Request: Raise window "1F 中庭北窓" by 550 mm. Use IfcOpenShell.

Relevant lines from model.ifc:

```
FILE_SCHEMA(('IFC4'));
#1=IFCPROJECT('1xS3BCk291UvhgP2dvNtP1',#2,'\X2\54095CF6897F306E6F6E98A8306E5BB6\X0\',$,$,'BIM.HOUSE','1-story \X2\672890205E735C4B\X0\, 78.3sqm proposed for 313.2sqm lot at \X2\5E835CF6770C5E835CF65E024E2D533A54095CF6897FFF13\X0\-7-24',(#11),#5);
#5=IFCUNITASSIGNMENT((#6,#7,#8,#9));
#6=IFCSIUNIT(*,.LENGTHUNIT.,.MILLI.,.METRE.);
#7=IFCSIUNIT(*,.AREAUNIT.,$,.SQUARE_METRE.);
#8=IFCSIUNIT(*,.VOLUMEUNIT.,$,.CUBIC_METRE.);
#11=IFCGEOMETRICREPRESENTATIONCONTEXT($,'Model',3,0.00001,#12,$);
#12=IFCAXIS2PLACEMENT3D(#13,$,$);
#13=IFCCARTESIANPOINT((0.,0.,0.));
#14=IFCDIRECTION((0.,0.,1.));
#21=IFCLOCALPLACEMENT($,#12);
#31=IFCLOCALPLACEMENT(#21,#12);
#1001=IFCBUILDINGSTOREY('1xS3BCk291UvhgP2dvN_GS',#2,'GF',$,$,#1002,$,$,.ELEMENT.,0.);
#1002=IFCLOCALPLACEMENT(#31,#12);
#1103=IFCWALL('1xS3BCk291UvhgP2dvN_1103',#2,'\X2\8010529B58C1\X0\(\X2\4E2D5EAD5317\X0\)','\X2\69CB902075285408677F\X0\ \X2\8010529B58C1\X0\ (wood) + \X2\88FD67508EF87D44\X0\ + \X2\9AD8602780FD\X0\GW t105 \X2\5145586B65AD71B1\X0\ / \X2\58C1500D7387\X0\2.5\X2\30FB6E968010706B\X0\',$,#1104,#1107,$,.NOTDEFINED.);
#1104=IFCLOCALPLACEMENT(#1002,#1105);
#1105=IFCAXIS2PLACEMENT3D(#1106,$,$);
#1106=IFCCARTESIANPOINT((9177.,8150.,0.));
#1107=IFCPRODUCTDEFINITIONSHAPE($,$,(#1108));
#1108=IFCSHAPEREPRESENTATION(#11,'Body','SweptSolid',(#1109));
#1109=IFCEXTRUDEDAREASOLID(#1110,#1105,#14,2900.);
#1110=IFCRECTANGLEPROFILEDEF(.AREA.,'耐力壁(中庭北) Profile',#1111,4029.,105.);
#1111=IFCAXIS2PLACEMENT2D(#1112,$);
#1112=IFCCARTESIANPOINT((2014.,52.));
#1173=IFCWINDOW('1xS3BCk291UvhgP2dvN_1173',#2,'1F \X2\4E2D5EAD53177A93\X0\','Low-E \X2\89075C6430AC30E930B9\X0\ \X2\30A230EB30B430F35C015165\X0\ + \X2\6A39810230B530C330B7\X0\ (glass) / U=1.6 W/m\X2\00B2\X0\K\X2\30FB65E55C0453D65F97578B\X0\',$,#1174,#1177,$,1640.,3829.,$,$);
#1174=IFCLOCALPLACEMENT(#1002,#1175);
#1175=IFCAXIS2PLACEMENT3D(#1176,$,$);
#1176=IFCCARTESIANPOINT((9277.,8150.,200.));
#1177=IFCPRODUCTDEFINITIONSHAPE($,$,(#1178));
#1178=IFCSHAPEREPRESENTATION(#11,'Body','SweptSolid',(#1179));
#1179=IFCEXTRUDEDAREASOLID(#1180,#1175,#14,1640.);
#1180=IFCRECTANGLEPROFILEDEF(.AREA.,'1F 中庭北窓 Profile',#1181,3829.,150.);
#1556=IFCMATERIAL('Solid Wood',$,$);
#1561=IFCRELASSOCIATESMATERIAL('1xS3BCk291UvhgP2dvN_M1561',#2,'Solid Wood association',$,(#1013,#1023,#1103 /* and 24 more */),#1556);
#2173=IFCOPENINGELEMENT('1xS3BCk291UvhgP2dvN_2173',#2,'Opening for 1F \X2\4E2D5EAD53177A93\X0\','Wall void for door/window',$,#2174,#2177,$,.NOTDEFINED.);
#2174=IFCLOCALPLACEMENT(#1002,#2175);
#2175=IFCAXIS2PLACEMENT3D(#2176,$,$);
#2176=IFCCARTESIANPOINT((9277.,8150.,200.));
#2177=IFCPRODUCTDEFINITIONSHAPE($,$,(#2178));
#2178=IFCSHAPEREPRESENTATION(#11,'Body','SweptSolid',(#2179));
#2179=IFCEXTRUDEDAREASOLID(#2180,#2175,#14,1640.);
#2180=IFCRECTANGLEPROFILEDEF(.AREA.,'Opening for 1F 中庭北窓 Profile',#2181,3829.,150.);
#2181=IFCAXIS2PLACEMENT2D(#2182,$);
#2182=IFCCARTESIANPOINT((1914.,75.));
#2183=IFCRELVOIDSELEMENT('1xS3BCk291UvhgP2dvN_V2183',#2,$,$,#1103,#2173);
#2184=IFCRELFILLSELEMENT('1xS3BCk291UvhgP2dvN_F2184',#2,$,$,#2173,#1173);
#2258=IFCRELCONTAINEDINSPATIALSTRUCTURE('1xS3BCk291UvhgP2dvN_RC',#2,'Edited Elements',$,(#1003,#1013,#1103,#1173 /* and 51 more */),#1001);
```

```python
import numpy as np
import ifcopenshell
import ifcopenshell.api.geometry
import ifcopenshell.util.placement
import ifcopenshell.util.unit

model = ifcopenshell.open("model.ifc")
unit_scale = ifcopenshell.util.unit.calculate_unit_scale(model)

window = model.by_guid("1xS3BCk291UvhgP2dvN_1173")
opening = window.FillsVoids[0].RelatingOpeningElement
dz = 550.0

shift = np.array([0.0, 0.0, dz])
# The window is not placed relative to its opening, so move both.
for product in (opening, window):
    matrix = ifcopenshell.util.placement.get_local_placement(product.ObjectPlacement)
    matrix[:3, 3] += shift
    ifcopenshell.api.geometry.edit_object_placement(model, product=product, matrix=matrix, is_si=False)

print(f"moved by {dz * unit_scale:+.3f} m")

model.write("model_rev.ifc")
```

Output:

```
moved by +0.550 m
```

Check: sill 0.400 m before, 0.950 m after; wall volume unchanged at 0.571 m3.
